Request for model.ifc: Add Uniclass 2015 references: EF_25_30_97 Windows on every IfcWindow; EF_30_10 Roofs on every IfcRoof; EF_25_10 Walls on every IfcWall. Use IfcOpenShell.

First a look at what the model holds.

```python
import ifcopenshell

model = ifcopenshell.open("model.ifc")
print(model.schema)
print("classifications:", [c.Name for c in model.by_type("IfcClassification")])
for ifc_class in ("IfcDoor", "IfcRoof", "IfcStair", "IfcWall", "IfcWindow"):
    print(ifc_class, len(model.by_type(ifc_class)))
```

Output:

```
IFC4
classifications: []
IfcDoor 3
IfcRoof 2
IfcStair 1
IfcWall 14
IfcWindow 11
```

```python
import ifcopenshell
import ifcopenshell.api.classification

model = ifcopenshell.open("model.ifc")

system = ifcopenshell.api.classification.add_classification(model, classification="Uniclass 2015")

codes = {
    "IfcWindow": ("EF_25_30_97", "Windows"),
    "IfcRoof": ("EF_30_10", "Roofs"),
    "IfcWall": ("EF_25_10", "Walls"),
}
for ifc_class, (code, name) in codes.items():
    products = model.by_type(ifc_class)
    ifcopenshell.api.classification.add_reference(
        model, products=products, classification=system, identification=code, name=name
    )
    print(code, len(products))

model.write("model_v2.ifc")
```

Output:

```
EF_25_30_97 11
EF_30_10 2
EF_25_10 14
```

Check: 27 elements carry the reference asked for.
